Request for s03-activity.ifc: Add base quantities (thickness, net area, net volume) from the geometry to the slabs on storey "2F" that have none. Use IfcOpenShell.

First a look at what the model holds.

```python
import ifcopenshell
import ifcopenshell.util.element
import ifcopenshell.util.unit

model = ifcopenshell.open("s03-activity.ifc")
print(model.schema)
for unit_type in ("LENGTHUNIT", "AREAUNIT", "VOLUMEUNIT"):
    print(unit_type, ifcopenshell.util.unit.calculate_unit_scale(model, unit_type))
storey = next(s for s in model.by_type("IfcBuildingStorey") if s.Name == "2F")
slabs = [e for e in ifcopenshell.util.element.get_decomposition(storey) if e.is_a("IfcSlab")]
for e in sorted(slabs, key=lambda e: e.id()):
    print(e.id(), e.is_a(), e.Name, list(ifcopenshell.util.element.get_psets(e, qtos_only=True)), sep=" | ")
```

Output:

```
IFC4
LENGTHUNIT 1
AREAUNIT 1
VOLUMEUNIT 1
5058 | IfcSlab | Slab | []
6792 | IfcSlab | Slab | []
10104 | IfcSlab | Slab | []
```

```python
import ifcopenshell
import ifcopenshell.api.pset
import ifcopenshell.geom
import ifcopenshell.util.element
import ifcopenshell.util.shape
import ifcopenshell.util.unit

model = ifcopenshell.open("s03-activity.ifc")
unit_scale = ifcopenshell.util.unit.calculate_unit_scale(model)
area_scale = ifcopenshell.util.unit.calculate_unit_scale(model, "AREAUNIT")
volume_scale = ifcopenshell.util.unit.calculate_unit_scale(model, "VOLUMEUNIT")
settings = ifcopenshell.geom.settings()

storey = next(s for s in model.by_type("IfcBuildingStorey") if s.Name == "2F")
slabs = [e for e in ifcopenshell.util.element.get_decomposition(storey) if e.is_a("IfcSlab")]

for e in sorted(slabs, key=lambda e: e.id()):
    if ifcopenshell.util.element.get_psets(e, qtos_only=True, should_inherit=False):
        continue
    # Geometry comes back in metres, in the element's own axes.
    shape = ifcopenshell.geom.create_shape(settings, e)
    values = {
        "Width": ifcopenshell.util.shape.get_z(shape.geometry) / unit_scale,
        "NetArea": ifcopenshell.util.shape.get_footprint_area(shape.geometry) / area_scale,
        "NetVolume": ifcopenshell.util.shape.get_volume(shape.geometry) / volume_scale,
    }
    qto = ifcopenshell.api.pset.add_qto(model, product=e, name="Qto_SlabBaseQuantities")
    ifcopenshell.api.pset.edit_qto(model, qto=qto, properties=values)
    print(e.id(), {k: round(v, 3) for k, v in values.items()})

model.write("s03-activity_v2.ifc")
```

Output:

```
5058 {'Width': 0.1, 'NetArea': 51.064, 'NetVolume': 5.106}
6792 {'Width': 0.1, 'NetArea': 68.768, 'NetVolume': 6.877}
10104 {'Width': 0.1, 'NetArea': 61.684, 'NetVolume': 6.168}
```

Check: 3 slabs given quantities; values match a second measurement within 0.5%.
